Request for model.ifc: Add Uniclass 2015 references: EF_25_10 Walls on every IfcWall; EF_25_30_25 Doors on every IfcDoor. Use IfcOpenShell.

First a look at what the model holds.

```python
import ifcopenshell

model = ifcopenshell.open("model.ifc")
print(model.schema)
print("classifications:", [c.Name for c in model.by_type("IfcClassification")])
for ifc_class in ("IfcDoor", "IfcRoof", "IfcStair", "IfcWall", "IfcWindow"):
    print(ifc_class, len(model.by_type(ifc_class)))
```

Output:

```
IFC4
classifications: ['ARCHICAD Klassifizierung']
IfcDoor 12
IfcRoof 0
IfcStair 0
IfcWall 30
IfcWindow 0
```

```python
import ifcopenshell
import ifcopenshell.api.classification

model = ifcopenshell.open("model.ifc")

system = ifcopenshell.api.classification.add_classification(model, classification="Uniclass 2015")

codes = {
    "IfcWall": ("EF_25_10", "Walls"),
    "IfcDoor": ("EF_25_30_25", "Doors"),
}
for ifc_class, (code, name) in codes.items():
    products = model.by_type(ifc_class)
    ifcopenshell.api.classification.add_reference(
        model, products=products, classification=system, identification=code, name=name
    )
    print(code, len(products))

model.write("model-out.ifc")
```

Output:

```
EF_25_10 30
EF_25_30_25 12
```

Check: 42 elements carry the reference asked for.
